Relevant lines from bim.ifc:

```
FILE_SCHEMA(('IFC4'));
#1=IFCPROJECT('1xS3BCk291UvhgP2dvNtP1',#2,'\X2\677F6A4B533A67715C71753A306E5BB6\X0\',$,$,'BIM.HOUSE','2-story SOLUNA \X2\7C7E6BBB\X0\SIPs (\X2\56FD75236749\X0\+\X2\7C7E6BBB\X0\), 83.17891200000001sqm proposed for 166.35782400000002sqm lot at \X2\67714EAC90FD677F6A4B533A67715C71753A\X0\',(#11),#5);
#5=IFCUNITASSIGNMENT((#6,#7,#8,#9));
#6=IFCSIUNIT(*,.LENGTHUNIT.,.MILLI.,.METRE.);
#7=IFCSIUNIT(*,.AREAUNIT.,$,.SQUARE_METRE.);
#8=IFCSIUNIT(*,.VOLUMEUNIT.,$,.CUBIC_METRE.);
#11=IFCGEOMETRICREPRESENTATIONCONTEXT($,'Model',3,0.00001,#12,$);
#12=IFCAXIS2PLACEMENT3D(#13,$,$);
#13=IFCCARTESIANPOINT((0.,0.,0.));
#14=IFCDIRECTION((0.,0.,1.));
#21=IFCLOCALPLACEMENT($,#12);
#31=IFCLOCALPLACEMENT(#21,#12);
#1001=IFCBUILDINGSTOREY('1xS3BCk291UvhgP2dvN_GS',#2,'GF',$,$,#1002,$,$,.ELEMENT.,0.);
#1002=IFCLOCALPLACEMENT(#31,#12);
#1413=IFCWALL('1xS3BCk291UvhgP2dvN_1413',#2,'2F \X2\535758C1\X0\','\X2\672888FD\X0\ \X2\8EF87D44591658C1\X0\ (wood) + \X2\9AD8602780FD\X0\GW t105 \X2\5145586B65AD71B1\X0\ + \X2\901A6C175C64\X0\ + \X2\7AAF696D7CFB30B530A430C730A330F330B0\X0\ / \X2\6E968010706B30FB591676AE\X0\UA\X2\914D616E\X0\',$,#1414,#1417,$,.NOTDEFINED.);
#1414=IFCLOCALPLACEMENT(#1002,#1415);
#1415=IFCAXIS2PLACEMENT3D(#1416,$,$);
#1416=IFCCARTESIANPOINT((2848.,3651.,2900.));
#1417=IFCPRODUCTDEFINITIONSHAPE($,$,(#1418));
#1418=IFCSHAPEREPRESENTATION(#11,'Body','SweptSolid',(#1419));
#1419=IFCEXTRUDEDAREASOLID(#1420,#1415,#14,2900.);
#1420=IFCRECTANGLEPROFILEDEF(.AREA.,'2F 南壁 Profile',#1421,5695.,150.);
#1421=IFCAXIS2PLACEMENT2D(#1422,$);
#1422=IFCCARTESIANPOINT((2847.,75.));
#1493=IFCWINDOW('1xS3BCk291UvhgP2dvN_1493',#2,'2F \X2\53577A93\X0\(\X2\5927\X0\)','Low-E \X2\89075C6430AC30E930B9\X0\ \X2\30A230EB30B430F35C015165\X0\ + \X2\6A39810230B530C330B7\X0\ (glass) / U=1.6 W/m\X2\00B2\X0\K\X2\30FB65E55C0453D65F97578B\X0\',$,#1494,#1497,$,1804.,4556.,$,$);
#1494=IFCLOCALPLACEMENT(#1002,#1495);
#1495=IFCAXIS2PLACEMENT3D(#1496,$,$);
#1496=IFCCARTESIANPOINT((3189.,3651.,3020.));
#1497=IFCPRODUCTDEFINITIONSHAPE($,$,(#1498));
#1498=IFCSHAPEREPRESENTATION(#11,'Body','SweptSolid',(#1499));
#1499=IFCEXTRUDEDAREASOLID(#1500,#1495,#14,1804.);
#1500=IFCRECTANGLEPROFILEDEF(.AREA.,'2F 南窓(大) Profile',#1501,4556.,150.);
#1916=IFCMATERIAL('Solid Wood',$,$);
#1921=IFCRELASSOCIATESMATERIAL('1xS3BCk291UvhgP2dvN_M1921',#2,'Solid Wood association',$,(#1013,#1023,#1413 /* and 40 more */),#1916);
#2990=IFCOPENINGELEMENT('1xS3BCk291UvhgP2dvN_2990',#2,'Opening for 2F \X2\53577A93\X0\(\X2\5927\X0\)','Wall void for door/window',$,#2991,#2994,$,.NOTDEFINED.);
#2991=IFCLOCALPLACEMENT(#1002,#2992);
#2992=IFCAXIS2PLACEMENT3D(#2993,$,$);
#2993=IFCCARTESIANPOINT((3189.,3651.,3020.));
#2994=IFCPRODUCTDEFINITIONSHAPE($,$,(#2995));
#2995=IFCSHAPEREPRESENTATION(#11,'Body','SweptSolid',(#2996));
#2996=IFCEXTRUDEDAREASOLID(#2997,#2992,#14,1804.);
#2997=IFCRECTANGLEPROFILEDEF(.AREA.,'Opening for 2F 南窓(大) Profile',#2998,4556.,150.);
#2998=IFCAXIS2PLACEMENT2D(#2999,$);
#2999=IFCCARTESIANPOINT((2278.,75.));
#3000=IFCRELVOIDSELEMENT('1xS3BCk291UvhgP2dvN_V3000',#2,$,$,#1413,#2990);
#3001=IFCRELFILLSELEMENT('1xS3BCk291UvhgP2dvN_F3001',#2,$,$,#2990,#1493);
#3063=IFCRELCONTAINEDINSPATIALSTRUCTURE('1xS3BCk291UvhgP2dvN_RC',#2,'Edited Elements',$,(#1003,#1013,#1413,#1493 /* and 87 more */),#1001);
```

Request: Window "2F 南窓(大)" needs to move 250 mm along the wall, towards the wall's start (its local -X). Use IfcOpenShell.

```python
import ifcopenshell
import ifcopenshell.api.geometry
import ifcopenshell.util.placement

model = ifcopenshell.open("bim.ifc")

window = model.by_guid("1xS3BCk291UvhgP2dvN_1493")
opening = window.FillsVoids[0].RelatingOpeningElement
wall = opening.VoidsElements[0].RelatingBuildingElement

wall_matrix = ifcopenshell.util.placement.get_local_placement(wall.ObjectPlacement)
shift = wall_matrix[:3, 0] * -250.0
before = ifcopenshell.util.placement.get_local_placement(window.ObjectPlacement)[:3, 3].copy()

# The window is not placed relative to its opening, so move both.
for product in (opening, window):
    matrix = ifcopenshell.util.placement.get_local_placement(product.ObjectPlacement)
    matrix[:3, 3] += shift
    ifcopenshell.api.geometry.edit_object_placement(model, product=product, matrix=matrix, is_si=False)

after = ifcopenshell.util.placement.get_local_placement(window.ObjectPlacement)[:3, 3]
print("window moved by", (after - before).round(3) + 0.0)

model.write("bim_edited.ifc")
```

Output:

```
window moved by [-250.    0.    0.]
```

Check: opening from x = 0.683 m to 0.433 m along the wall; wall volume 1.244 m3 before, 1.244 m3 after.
